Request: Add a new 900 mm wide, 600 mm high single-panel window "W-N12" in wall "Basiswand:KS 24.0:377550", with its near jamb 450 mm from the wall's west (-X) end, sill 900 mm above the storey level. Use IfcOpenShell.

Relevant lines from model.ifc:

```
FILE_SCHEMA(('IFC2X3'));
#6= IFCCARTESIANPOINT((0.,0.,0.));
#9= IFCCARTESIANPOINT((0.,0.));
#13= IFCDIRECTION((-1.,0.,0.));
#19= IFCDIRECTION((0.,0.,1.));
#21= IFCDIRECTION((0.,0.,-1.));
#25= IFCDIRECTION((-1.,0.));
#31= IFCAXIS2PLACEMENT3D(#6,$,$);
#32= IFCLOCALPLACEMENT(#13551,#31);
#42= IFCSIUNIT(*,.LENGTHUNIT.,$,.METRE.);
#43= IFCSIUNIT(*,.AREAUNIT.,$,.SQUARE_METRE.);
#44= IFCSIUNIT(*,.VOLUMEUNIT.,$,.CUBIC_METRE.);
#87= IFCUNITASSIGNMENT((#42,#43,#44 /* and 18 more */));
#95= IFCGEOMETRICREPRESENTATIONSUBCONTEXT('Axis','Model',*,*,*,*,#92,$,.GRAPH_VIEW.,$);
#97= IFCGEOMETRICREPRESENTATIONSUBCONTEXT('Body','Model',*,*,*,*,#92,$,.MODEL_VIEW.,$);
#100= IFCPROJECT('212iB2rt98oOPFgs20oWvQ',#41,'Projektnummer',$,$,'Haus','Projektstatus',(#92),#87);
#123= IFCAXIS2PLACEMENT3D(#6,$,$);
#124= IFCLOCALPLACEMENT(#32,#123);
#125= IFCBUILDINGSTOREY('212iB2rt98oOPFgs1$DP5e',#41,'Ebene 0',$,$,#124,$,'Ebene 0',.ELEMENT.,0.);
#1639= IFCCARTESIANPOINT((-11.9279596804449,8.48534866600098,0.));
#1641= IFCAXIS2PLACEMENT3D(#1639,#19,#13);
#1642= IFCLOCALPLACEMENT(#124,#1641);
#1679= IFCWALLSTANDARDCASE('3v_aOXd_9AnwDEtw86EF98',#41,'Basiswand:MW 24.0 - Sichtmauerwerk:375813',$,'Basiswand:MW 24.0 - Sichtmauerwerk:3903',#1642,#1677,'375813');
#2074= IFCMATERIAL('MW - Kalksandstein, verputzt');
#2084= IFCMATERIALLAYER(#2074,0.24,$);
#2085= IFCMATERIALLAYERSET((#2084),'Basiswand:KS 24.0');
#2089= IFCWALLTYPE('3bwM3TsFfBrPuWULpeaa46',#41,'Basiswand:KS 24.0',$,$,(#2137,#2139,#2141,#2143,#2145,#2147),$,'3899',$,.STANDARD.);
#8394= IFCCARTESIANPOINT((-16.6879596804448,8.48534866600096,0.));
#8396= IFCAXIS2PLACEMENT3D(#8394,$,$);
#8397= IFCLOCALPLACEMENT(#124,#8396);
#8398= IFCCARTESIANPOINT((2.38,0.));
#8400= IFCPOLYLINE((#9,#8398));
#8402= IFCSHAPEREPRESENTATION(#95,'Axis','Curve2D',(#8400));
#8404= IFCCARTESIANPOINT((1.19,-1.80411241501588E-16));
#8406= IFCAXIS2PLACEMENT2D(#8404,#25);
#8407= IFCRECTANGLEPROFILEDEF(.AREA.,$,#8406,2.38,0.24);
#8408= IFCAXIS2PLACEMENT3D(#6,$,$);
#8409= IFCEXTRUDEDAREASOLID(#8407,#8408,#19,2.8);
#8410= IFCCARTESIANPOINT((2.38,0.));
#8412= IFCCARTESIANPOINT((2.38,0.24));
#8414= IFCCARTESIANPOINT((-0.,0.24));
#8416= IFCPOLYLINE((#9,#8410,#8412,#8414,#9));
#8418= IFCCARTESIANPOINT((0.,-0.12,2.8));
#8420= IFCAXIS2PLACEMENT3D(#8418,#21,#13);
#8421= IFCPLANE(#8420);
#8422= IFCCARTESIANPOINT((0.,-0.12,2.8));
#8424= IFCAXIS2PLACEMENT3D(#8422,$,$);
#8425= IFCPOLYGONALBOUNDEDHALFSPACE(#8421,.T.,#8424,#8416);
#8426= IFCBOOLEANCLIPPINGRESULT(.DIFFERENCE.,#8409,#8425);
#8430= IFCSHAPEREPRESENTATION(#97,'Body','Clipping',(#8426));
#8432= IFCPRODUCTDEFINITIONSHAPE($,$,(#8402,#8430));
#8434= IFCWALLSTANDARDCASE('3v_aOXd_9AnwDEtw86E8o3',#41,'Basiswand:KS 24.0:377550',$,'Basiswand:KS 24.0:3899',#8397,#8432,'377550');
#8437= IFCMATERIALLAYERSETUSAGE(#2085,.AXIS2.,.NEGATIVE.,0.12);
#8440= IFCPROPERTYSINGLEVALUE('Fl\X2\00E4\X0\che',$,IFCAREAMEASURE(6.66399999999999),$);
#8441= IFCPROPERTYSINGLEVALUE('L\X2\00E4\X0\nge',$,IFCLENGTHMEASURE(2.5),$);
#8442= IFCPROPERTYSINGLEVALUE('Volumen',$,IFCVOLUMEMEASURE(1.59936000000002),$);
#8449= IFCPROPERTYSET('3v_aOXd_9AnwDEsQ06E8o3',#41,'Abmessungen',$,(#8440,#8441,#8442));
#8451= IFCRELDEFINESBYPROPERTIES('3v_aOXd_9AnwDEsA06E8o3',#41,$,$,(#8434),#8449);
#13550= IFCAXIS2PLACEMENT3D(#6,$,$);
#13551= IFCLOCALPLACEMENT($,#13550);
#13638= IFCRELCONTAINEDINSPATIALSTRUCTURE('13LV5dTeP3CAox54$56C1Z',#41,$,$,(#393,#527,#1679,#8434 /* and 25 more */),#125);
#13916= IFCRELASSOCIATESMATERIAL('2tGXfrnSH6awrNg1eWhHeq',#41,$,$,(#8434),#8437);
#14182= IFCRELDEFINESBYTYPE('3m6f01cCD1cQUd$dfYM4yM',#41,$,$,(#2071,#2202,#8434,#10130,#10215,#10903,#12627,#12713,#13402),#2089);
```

```python
import numpy as np
import ifcopenshell
import ifcopenshell.api.feature
import ifcopenshell.api.geometry
import ifcopenshell.api.pset
import ifcopenshell.api.root
import ifcopenshell.api.spatial
import ifcopenshell.api.type
import ifcopenshell.geom
import ifcopenshell.util.element
import ifcopenshell.util.placement
import ifcopenshell.util.representation
import ifcopenshell.util.shape
import ifcopenshell.util.unit

model = ifcopenshell.open("model.ifc")
unit_scale = ifcopenshell.util.unit.calculate_unit_scale(model)
area_scale = ifcopenshell.util.unit.calculate_unit_scale(model, "AREAUNIT")
volume_scale = ifcopenshell.util.unit.calculate_unit_scale(model, "VOLUMEUNIT")
settings = ifcopenshell.geom.settings()


def volume(element):
    """Net volume in cubic metres, openings subtracted."""
    shape = ifcopenshell.geom.create_shape(settings, element)
    return ifcopenshell.util.shape.get_volume(shape.geometry)


wall = model.by_guid("3v_aOXd_9AnwDEtw86E8o3")
storey = ifcopenshell.util.element.get_container(wall, ifc_class="IfcBuildingStorey")
context = ifcopenshell.util.representation.get_context(model, "Model", "Body", "MODEL_VIEW")
before = volume(wall)

width, height, from_end, sill = 0.9, 0.6, 0.45, 0.9  # metres

# The wall runs along its own X axis, and the end named is its -X end.
wall_shape = ifcopenshell.geom.create_shape(settings, wall)
x, y, z = ifcopenshell.util.shape.get_vertices(wall_shape.geometry).T
start = x.min() + from_end
face, thickness = float(y.min()), float(y.max() - y.min())
wall_matrix = ifcopenshell.util.placement.get_local_placement(wall.ObjectPlacement)
level = ifcopenshell.util.placement.get_local_placement(storey.ObjectPlacement)[2, 3]


def in_wall(x, y):
    """Placement at x, y metres in the wall's axes, at sill height."""
    matrix = wall_matrix.copy()
    matrix[:, 3] = wall_matrix @ np.array([x / unit_scale, y / unit_scale, 0.0, 1.0])
    matrix[2, 3] = level + sill / unit_scale
    return matrix


# Opening: a box that overshoots both wall faces by 50 mm.
opening = ifcopenshell.api.root.create_entity(model, ifc_class="IfcOpeningElement")
box = ifcopenshell.api.geometry.add_wall_representation(
    model, context=context, length=width, height=height, thickness=thickness + 0.1
)
ifcopenshell.api.geometry.assign_representation(model, product=opening, representation=box)
ifcopenshell.api.geometry.edit_object_placement(model, product=opening, matrix=in_wall(start, face - 0.05), is_si=False)
ifcopenshell.api.feature.add_feature(model, feature=opening, element=wall)

window = ifcopenshell.api.root.create_entity(model, ifc_class="IfcWindow", name="W-N12")
window.OverallWidth, window.OverallHeight = width / unit_scale, height / unit_scale
body = ifcopenshell.api.geometry.add_window_representation(
    model,
    context=context,
    overall_width=window.OverallWidth,
    overall_height=window.OverallHeight,
    partition_type="SINGLE_PANEL",
)
ifcopenshell.api.geometry.assign_representation(model, product=window, representation=body)
ifcopenshell.api.spatial.assign_container(model, products=[window], relating_structure=storey)
fills = ifcopenshell.api.feature.add_filling(model, opening=opening, element=window)
fills.OwnerHistory = window.OwnerHistory  # required in IFC2X3

# IFC2X3 keeps the operation on the window style.
style = ifcopenshell.api.root.create_entity(model, ifc_class="IfcWindowStyle", name="W-N12")
style.OperationType, style.ConstructionType = "SINGLE_PANEL", "NOTDEFINED"
style.ParameterTakesPrecedence = style.Sizeable = False
ifcopenshell.api.type.assign_type(model, related_objects=[window], relating_type=style)

# Centre the window in the wall's thickness.
ifcopenshell.api.geometry.edit_object_placement(model, product=window, matrix=in_wall(start, face), is_si=False)
window_shape = ifcopenshell.geom.create_shape(settings, window)
depth = ifcopenshell.util.shape.get_vertices(window_shape.geometry)[:, 1]
offset = face + thickness / 2 - (depth.min() + depth.max()) / 2
ifcopenshell.api.geometry.edit_object_placement(model, product=window, matrix=in_wall(start, offset), is_si=False)

after = volume(wall)

# Update the wall's stored quantities.
pset = model.by_id(ifcopenshell.util.element.get_pset(wall, "Abmessungen", should_inherit=False)["id"])
ifcopenshell.api.pset.edit_pset(model, pset=pset, properties={
    "Fläche": model.create_entity("IfcAreaMeasure", after / thickness / area_scale),
    "Volumen": model.create_entity("IfcVolumeMeasure", after / volume_scale),
})

print(f"wall volume {before:.3f} -> {after:.3f} m3")

model.write("model-out.ifc")
```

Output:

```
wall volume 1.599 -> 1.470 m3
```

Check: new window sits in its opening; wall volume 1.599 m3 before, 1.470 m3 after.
